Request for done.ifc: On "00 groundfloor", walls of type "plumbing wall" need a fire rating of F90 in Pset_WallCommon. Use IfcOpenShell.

First a look at what the model holds.

```python
import ifcopenshell
import ifcopenshell.util.element

model = ifcopenshell.open("done.ifc")
print(model.schema)
storey = next(s for s in model.by_type("IfcBuildingStorey") if s.Name == "00 groundfloor")
walls = [e for e in ifcopenshell.util.element.get_decomposition(storey) if e.is_a("IfcWall")]
seen = {}
for e in walls:
    element_type = ifcopenshell.util.element.get_type(e)
    key = (element_type.Name if element_type != e and element_type else None, ifcopenshell.util.element.get_pset(e, "Pset_WallCommon", "FireRating"))
    seen[key] = seen.get(key, 0) + 1
for (name, value), count in sorted(seen.items(), key=str):
    print(count, "x", name, "|", value)
```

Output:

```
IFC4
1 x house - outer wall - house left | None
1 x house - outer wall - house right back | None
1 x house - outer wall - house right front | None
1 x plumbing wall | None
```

```python
import ifcopenshell
import ifcopenshell.api.pset
import ifcopenshell.util.element

model = ifcopenshell.open("done.ifc")

storey = next(s for s in model.by_type("IfcBuildingStorey") if s.Name == "00 groundfloor")
walls = [e for e in ifcopenshell.util.element.get_decomposition(storey) if e.is_a("IfcWall")]

count = 0
for e in walls:
    element_type = ifcopenshell.util.element.get_type(e)
    if element_type in (None, e) or element_type.Name != "plumbing wall":
        continue
    # add_pset returns the element's existing set when there is one.
    pset = ifcopenshell.api.pset.add_pset(model, product=e, name="Pset_WallCommon")
    ifcopenshell.api.pset.edit_pset(model, pset=pset, properties={"FireRating": "F90"})
    count += 1

print(count, "walls updated")

model.write("done_rev.ifc")
```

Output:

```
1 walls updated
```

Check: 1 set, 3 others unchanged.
